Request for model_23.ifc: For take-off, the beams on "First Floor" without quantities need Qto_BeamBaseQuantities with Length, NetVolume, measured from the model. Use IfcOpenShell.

First a look at what the model holds.

```python
import ifcopenshell
import ifcopenshell.util.element
import ifcopenshell.util.unit

model = ifcopenshell.open("model_23.ifc")
print(model.schema)
for unit_type in ("LENGTHUNIT", "AREAUNIT", "VOLUMEUNIT"):
    print(unit_type, ifcopenshell.util.unit.calculate_unit_scale(model, unit_type))
storey = next(s for s in model.by_type("IfcBuildingStorey") if s.Name == "First Floor")
beams = [e for e in ifcopenshell.util.element.get_decomposition(storey) if e.is_a("IfcBeam")]
for e in sorted(beams, key=lambda e: e.id()):
    print(e.id(), e.is_a(), e.Name, list(ifcopenshell.util.element.get_psets(e, qtos_only=True)), sep=" | ")
```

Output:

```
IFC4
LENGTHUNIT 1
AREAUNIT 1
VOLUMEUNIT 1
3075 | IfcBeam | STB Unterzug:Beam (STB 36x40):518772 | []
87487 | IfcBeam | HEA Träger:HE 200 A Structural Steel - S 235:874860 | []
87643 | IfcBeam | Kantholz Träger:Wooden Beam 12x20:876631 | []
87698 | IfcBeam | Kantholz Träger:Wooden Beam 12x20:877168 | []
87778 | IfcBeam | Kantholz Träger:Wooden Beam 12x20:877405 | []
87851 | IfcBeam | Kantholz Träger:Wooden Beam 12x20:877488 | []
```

```python
import ifcopenshell
import ifcopenshell.api.pset
import ifcopenshell.geom
import ifcopenshell.util.element
import ifcopenshell.util.shape
import ifcopenshell.util.unit

model = ifcopenshell.open("model_23.ifc")
unit_scale = ifcopenshell.util.unit.calculate_unit_scale(model)
volume_scale = ifcopenshell.util.unit.calculate_unit_scale(model, "VOLUMEUNIT")
settings = ifcopenshell.geom.settings()

storey = next(s for s in model.by_type("IfcBuildingStorey") if s.Name == "First Floor")
beams = [e for e in ifcopenshell.util.element.get_decomposition(storey) if e.is_a("IfcBeam")]

for e in sorted(beams, key=lambda e: e.id()):
    if ifcopenshell.util.element.get_psets(e, qtos_only=True, should_inherit=False):
        continue
    # Geometry comes back in metres, in the element's own axes.
    shape = ifcopenshell.geom.create_shape(settings, e)
    values = {
        "Length": ifcopenshell.util.shape.get_max_xyz(shape.geometry) / unit_scale,
        "NetVolume": ifcopenshell.util.shape.get_volume(shape.geometry) / volume_scale,
    }
    qto = ifcopenshell.api.pset.add_qto(model, product=e, name="Qto_BeamBaseQuantities")
    ifcopenshell.api.pset.edit_qto(model, qto=qto, properties=values)
    print(e.id(), {k: round(v, 3) for k, v in values.items()})

model.write("model_23-out.ifc")
```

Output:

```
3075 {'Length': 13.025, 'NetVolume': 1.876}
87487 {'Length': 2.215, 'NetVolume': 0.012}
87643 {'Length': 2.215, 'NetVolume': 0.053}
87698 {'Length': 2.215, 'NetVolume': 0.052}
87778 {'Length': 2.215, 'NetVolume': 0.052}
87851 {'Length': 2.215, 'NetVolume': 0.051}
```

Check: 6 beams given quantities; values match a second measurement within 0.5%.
